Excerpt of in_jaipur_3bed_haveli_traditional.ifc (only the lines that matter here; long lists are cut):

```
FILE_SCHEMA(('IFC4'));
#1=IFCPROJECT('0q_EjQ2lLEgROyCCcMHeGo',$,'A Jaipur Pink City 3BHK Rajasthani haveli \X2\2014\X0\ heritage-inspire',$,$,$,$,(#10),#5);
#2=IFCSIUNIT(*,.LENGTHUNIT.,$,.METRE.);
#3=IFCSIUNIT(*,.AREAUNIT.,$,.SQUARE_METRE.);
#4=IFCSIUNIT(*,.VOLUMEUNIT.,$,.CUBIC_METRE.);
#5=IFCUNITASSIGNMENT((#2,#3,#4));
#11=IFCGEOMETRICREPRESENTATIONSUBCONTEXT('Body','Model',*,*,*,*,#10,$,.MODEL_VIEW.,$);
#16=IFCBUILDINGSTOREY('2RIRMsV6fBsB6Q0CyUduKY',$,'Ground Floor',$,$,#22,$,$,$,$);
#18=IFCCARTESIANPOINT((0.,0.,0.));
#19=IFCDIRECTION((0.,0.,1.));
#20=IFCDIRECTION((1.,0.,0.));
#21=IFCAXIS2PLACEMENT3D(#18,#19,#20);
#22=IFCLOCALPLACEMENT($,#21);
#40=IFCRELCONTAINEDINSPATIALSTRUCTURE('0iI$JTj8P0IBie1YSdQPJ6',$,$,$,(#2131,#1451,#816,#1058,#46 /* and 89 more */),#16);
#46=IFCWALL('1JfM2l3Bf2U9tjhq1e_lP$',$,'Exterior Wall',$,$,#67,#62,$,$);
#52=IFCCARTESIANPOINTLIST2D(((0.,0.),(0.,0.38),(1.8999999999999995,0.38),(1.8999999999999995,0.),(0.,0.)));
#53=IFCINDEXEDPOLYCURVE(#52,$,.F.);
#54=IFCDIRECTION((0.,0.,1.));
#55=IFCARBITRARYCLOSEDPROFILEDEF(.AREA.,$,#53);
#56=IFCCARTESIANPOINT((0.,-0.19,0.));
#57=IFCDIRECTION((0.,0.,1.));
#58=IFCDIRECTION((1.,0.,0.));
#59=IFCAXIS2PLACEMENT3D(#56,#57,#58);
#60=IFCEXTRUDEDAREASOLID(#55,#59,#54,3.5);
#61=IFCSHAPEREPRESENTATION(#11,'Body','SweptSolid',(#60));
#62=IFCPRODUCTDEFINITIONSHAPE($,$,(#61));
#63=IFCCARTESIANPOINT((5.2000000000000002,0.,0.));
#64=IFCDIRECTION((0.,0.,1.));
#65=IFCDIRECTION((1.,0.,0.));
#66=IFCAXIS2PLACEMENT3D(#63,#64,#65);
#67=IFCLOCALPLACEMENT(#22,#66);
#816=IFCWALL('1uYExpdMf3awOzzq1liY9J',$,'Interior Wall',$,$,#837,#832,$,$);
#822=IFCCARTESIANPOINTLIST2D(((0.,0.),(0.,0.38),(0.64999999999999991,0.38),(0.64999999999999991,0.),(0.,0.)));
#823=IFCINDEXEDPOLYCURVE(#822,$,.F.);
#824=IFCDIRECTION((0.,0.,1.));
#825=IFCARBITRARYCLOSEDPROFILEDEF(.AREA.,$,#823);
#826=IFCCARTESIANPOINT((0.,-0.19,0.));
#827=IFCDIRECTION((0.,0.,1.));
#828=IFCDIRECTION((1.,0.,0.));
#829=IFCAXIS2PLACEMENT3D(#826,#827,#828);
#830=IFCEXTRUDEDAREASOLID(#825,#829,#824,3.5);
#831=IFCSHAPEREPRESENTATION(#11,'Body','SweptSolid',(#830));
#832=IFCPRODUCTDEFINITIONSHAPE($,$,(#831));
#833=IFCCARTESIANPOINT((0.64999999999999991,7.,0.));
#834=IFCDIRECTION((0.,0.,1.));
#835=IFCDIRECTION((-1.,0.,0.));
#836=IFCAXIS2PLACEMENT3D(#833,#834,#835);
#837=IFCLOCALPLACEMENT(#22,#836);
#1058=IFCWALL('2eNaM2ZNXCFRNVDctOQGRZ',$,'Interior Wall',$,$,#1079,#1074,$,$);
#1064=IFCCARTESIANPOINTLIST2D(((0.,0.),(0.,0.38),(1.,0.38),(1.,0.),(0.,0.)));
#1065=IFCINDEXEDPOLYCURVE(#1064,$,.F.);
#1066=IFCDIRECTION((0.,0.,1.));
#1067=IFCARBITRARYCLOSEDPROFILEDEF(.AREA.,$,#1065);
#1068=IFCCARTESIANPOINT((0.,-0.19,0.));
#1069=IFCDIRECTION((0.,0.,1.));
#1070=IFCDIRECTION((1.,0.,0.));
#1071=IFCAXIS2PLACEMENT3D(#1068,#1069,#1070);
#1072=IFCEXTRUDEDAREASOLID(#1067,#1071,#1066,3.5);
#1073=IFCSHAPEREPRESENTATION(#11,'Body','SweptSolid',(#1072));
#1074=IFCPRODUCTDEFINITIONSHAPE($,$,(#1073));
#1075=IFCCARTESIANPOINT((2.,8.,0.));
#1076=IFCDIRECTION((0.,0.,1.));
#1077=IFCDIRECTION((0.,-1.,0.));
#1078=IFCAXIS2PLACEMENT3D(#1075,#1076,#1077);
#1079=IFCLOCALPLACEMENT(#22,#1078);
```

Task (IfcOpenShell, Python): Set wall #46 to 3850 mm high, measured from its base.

```python
import ifcopenshell
import ifcopenshell.geom
import ifcopenshell.util.representation
import ifcopenshell.util.shape
import ifcopenshell.util.unit

model = ifcopenshell.open("in_jaipur_3bed_haveli_traditional.ifc")
unit_scale = ifcopenshell.util.unit.calculate_unit_scale(model)
settings = ifcopenshell.geom.settings()


def volume(element):
    """Net volume in cubic metres, openings subtracted."""
    shape = ifcopenshell.geom.create_shape(settings, element)
    return ifcopenshell.util.shape.get_volume(shape.geometry)


wall = model.by_guid("1JfM2l3Bf2U9tjhq1e_lP$")
before = volume(wall)

body = ifcopenshell.util.representation.get_representation(wall, "Model", "Body")
solid = body.Items[0]
old_height = solid.Depth
solid.Depth = 3.85 / unit_scale
after = volume(wall)

print(f"height {old_height:g} -> {solid.Depth:g}, volume {before:.3f} -> {after:.3f} m3")

model.write("in_jaipur_3bed_haveli_traditional_v2.ifc")
```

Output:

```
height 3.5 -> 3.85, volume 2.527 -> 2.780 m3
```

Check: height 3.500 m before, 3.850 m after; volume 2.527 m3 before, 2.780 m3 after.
